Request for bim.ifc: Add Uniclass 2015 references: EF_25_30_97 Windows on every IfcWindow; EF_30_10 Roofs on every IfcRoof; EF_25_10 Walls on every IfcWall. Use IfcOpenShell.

First a look at what the model holds.

```python
import ifcopenshell

model = ifcopenshell.open("bim.ifc")
print(model.schema)
print("classifications:", [c.Name for c in model.by_type("IfcClassification")])
for ifc_class in ("IfcDoor", "IfcRoof", "IfcStair", "IfcWall", "IfcWindow"):
    print(ifc_class, len(model.by_type(ifc_class)))
```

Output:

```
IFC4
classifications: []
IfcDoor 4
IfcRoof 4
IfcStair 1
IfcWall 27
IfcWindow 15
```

```python
import ifcopenshell
import ifcopenshell.api.classification

model = ifcopenshell.open("bim.ifc")

system = ifcopenshell.api.classification.add_classification(model, classification="Uniclass 2015")

codes = {
    "IfcWindow": ("EF_25_30_97", "Windows"),
    "IfcRoof": ("EF_30_10", "Roofs"),
    "IfcWall": ("EF_25_10", "Walls"),
}
for ifc_class, (code, name) in codes.items():
    products = model.by_type(ifc_class)
    ifcopenshell.api.classification.add_reference(
        model, products=products, classification=system, identification=code, name=name
    )
    print(code, len(products))

model.write("bim_updated.ifc")
```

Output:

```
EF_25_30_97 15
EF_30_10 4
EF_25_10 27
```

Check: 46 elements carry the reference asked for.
